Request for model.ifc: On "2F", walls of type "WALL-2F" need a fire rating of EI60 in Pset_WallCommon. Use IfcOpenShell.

First a look at what the model holds.

```python
import ifcopenshell
import ifcopenshell.util.element

model = ifcopenshell.open("model.ifc")
print(model.schema)
storey = next(s for s in model.by_type("IfcBuildingStorey") if s.Name == "2F")
walls = [e for e in ifcopenshell.util.element.get_decomposition(storey) if e.is_a("IfcWall")]
seen = {}
for e in walls:
    element_type = ifcopenshell.util.element.get_type(e)
    key = (element_type.Name if element_type != e and element_type else None, ifcopenshell.util.element.get_pset(e, "Pset_WallCommon", "FireRating"))
    seen[key] = seen.get(key, 0) + 1
for (name, value), count in sorted(seen.items(), key=str):
    print(count, "x", name, "|", value)
```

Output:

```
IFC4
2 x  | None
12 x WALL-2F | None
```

```python
import ifcopenshell
import ifcopenshell.api.pset
import ifcopenshell.util.element

model = ifcopenshell.open("model.ifc")

storey = next(s for s in model.by_type("IfcBuildingStorey") if s.Name == "2F")
walls = [e for e in ifcopenshell.util.element.get_decomposition(storey) if e.is_a("IfcWall")]

count = 0
for e in walls:
    element_type = ifcopenshell.util.element.get_type(e)
    if element_type in (None, e) or element_type.Name != "WALL-2F":
        continue
    # add_pset returns the element's existing set when there is one.
    pset = ifcopenshell.api.pset.add_pset(model, product=e, name="Pset_WallCommon")
    ifcopenshell.api.pset.edit_pset(model, pset=pset, properties={"FireRating": "EI60"})
    count += 1

print(count, "walls updated")

model.write("model_rev.ifc")
```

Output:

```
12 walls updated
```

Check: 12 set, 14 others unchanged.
